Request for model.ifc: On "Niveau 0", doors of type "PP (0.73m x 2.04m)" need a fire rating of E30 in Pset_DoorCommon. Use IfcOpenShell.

First a look at what the model holds.

```python
import ifcopenshell
import ifcopenshell.util.element

model = ifcopenshell.open("model.ifc")
print(model.schema)
storey = next(s for s in model.by_type("IfcBuildingStorey") if s.Name == "Niveau 0")
doors = [e for e in ifcopenshell.util.element.get_decomposition(storey) if e.is_a("IfcDoor")]
seen = {}
for e in doors:
    element_type = ifcopenshell.util.element.get_type(e)
    key = (element_type.Name if element_type != e and element_type else None, ifcopenshell.util.element.get_pset(e, "Pset_DoorCommon", "FireRating"))
    seen[key] = seen.get(key, 0) + 1
for (name, value), count in sorted(seen.items(), key=str):
    print(count, "x", name, "|", value)
```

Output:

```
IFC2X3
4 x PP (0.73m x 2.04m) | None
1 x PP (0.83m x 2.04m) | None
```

```python
import ifcopenshell
import ifcopenshell.api.pset
import ifcopenshell.util.element

model = ifcopenshell.open("model.ifc")

storey = next(s for s in model.by_type("IfcBuildingStorey") if s.Name == "Niveau 0")
doors = [e for e in ifcopenshell.util.element.get_decomposition(storey) if e.is_a("IfcDoor")]

count = 0
for e in doors:
    element_type = ifcopenshell.util.element.get_type(e)
    if element_type in (None, e) or element_type.Name != "PP (0.73m x 2.04m)":
        continue
    # add_pset returns the element's existing set when there is one.
    pset = ifcopenshell.api.pset.add_pset(model, product=e, name="Pset_DoorCommon")
    ifcopenshell.api.pset.edit_pset(model, pset=pset, properties={"FireRating": "E30"})
    count += 1

print(count, "doors updated")

model.write("model-out.ifc")
```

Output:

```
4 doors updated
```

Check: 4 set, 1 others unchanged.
